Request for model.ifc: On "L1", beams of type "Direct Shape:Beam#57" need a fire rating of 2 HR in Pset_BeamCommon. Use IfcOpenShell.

First a look at what the model holds.

```python
import ifcopenshell
import ifcopenshell.util.element

model = ifcopenshell.open("model.ifc")
print(model.schema)
storey = next(s for s in model.by_type("IfcBuildingStorey") if s.Name == "L1")
beams = [e for e in ifcopenshell.util.element.get_decomposition(storey) if e.is_a("IfcBeam")]
seen = {}
for e in beams:
    element_type = ifcopenshell.util.element.get_type(e)
    key = (element_type.Name if element_type != e and element_type else None, ifcopenshell.util.element.get_pset(e, "Pset_BeamCommon", "FireRating"))
    seen[key] = seen.get(key, 0) + 1
for (name, value), count in sorted(seen.items(), key=str):
    print(count, "x", name, "|", value)
```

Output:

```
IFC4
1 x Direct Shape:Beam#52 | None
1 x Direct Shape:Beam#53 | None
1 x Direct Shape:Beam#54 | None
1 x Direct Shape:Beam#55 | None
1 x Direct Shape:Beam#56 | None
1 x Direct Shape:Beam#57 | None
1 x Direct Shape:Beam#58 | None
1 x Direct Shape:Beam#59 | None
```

```python
import ifcopenshell
import ifcopenshell.api.pset
import ifcopenshell.util.element

model = ifcopenshell.open("model.ifc")

storey = next(s for s in model.by_type("IfcBuildingStorey") if s.Name == "L1")
beams = [e for e in ifcopenshell.util.element.get_decomposition(storey) if e.is_a("IfcBeam")]

count = 0
for e in beams:
    element_type = ifcopenshell.util.element.get_type(e)
    if element_type in (None, e) or element_type.Name != "Direct Shape:Beam#57":
        continue
    # add_pset returns the element's existing set when there is one.
    pset = ifcopenshell.api.pset.add_pset(model, product=e, name="Pset_BeamCommon")
    ifcopenshell.api.pset.edit_pset(model, pset=pset, properties={"FireRating": "2 HR"})
    count += 1

print(count, "beams updated")

model.write("model-out.ifc")
```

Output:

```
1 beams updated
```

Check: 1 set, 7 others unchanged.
